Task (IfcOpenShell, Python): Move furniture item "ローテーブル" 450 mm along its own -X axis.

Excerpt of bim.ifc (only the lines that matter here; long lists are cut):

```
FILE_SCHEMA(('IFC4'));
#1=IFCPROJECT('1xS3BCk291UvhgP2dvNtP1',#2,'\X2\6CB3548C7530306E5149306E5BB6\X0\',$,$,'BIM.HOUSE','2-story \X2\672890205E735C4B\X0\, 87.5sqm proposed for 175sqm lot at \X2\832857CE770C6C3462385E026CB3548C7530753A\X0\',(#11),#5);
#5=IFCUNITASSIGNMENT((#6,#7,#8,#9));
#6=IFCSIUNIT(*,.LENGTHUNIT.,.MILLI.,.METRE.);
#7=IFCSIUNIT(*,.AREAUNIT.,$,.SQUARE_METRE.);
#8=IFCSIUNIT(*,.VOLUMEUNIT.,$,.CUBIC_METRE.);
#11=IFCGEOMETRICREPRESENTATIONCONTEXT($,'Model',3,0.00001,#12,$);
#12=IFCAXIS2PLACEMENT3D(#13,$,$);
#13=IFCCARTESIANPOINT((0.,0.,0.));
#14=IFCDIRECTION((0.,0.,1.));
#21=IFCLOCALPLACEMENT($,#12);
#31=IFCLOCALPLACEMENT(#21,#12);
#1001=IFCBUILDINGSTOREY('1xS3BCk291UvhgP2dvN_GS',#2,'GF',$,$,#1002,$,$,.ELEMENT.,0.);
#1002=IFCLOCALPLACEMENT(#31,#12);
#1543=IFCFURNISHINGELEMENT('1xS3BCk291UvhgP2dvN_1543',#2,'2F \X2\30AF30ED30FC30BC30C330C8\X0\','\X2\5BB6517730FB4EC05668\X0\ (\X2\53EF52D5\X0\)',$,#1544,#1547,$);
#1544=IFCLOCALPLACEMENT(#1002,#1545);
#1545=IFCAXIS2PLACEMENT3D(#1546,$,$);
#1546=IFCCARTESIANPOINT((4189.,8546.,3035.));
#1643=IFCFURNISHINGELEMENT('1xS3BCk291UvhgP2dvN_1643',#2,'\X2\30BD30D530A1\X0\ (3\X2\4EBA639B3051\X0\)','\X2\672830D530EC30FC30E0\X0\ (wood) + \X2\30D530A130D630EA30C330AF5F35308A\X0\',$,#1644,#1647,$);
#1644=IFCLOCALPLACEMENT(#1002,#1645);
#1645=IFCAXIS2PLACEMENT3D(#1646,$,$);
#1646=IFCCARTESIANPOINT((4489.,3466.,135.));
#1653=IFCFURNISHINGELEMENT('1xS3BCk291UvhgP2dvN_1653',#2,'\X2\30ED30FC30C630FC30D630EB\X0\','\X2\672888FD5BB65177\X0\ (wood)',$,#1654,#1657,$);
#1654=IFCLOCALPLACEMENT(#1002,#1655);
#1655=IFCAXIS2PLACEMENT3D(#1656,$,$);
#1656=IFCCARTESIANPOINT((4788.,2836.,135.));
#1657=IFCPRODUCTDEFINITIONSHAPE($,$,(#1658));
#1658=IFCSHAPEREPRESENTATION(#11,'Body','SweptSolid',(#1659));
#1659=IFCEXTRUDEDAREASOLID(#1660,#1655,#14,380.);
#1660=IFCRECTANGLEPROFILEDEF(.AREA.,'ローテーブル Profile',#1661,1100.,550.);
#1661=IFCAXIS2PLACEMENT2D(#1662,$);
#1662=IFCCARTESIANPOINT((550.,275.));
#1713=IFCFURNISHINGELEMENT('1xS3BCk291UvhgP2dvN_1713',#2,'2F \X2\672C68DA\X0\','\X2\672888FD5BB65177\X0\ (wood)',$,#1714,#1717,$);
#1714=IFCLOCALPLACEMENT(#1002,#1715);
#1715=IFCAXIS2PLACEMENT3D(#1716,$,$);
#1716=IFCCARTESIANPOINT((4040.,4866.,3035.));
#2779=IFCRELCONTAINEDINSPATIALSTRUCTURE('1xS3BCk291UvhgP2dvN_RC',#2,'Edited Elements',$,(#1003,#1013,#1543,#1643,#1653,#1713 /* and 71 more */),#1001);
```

```python
import ifcopenshell
import ifcopenshell.api.geometry
import ifcopenshell.util.placement
import ifcopenshell.util.unit

model = ifcopenshell.open("bim.ifc")
unit_scale = ifcopenshell.util.unit.calculate_unit_scale(model)

item = model.by_id(1653)
matrix = ifcopenshell.util.placement.get_local_placement(item.ObjectPlacement)
matrix[:3, 3] -= matrix[:3, 0] * 0.45 / unit_scale
ifcopenshell.api.geometry.edit_object_placement(model, product=item, matrix=matrix, is_si=False)

print(ifcopenshell.util.placement.get_local_placement(item.ObjectPlacement).round(3) + 0.0)

model.write("bim_edited.ifc")
```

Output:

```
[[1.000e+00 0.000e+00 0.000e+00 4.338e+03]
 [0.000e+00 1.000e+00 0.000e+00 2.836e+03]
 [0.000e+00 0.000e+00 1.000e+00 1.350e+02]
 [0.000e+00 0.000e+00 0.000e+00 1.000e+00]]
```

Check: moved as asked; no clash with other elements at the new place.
